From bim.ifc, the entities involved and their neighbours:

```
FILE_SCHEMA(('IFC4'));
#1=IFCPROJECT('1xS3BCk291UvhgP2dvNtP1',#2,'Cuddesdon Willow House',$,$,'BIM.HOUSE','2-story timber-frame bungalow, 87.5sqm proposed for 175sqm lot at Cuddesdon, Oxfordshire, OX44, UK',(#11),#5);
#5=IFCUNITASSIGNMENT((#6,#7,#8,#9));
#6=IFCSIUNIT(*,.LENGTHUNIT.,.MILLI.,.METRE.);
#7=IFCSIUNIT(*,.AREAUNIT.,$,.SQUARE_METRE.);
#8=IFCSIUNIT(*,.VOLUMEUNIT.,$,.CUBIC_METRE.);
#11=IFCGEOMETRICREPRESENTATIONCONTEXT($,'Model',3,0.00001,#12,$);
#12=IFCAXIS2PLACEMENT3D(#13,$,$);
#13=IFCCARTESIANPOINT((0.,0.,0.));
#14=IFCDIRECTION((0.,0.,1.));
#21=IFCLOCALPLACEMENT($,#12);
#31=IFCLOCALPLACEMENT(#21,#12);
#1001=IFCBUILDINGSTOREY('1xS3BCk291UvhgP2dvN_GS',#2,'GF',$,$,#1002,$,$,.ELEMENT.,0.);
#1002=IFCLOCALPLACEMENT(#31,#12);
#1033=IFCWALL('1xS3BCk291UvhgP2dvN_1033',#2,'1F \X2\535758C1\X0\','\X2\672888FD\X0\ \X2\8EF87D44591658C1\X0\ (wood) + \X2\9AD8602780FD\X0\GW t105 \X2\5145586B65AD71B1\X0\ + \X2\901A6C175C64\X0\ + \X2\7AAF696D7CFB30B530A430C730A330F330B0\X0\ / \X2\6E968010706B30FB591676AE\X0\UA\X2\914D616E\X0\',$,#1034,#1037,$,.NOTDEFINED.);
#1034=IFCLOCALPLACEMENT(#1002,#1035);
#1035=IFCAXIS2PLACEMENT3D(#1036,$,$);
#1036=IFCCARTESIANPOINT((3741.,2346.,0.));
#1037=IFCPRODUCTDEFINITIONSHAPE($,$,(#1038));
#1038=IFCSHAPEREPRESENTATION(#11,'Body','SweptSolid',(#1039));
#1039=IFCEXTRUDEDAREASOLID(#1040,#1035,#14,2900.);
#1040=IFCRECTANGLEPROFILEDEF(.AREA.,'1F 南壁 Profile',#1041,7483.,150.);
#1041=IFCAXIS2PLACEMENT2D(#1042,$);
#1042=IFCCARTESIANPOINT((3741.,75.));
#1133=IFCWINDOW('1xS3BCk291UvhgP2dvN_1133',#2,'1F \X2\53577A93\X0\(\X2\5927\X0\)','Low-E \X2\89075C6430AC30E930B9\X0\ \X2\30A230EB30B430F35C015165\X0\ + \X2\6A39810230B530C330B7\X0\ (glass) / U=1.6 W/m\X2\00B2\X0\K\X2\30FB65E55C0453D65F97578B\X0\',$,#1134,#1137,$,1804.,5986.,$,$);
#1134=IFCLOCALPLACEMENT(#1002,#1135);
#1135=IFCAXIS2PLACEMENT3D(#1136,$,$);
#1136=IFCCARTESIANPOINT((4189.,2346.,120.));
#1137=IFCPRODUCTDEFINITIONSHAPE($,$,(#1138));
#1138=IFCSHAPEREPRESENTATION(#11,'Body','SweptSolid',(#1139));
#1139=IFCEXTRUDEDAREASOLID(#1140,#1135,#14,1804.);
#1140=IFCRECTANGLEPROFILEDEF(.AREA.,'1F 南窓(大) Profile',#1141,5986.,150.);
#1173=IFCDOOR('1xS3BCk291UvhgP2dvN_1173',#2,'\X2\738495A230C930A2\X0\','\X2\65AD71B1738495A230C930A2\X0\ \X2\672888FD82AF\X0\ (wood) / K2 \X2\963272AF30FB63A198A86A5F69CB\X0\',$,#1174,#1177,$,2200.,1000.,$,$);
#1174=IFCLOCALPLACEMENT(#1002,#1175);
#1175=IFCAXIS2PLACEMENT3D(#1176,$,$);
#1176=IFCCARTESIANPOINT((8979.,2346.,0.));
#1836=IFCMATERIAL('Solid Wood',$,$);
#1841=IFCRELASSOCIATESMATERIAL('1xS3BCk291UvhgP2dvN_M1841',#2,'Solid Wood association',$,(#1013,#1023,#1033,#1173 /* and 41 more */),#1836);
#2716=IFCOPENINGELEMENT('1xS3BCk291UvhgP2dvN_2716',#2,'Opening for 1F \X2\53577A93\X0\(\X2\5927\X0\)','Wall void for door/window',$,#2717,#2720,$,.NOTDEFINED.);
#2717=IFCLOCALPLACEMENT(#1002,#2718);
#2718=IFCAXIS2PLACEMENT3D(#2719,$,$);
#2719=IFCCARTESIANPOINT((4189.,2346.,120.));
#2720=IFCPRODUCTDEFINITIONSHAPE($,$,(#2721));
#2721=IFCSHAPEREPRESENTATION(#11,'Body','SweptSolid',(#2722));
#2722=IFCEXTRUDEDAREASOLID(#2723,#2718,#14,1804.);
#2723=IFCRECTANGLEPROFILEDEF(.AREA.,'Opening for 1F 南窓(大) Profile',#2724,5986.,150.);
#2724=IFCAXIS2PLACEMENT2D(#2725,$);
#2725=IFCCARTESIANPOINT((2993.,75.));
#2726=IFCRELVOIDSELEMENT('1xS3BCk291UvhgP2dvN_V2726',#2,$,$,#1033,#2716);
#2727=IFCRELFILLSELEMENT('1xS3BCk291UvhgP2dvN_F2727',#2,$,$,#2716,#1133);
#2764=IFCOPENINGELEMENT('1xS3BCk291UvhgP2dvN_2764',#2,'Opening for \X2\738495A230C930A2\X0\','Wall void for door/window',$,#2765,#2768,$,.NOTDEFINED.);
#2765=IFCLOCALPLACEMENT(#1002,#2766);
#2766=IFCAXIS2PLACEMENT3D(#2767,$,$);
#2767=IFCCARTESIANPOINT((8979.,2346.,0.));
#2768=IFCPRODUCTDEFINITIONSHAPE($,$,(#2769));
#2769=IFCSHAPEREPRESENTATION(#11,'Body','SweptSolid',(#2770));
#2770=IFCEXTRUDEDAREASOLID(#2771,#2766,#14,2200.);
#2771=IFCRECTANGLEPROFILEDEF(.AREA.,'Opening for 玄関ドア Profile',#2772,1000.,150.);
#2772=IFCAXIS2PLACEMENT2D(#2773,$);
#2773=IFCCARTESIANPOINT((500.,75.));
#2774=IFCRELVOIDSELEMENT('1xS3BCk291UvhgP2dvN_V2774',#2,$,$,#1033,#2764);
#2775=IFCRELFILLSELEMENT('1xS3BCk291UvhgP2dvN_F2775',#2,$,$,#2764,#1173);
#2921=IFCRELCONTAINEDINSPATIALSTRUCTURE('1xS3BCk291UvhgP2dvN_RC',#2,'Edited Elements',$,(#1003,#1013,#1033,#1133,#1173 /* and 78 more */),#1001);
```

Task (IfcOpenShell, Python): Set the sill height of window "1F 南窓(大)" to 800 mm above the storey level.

```python
import numpy as np
import ifcopenshell
import ifcopenshell.api.geometry
import ifcopenshell.geom
import ifcopenshell.util.element
import ifcopenshell.util.placement
import ifcopenshell.util.shape
import ifcopenshell.util.unit

model = ifcopenshell.open("bim.ifc")
unit_scale = ifcopenshell.util.unit.calculate_unit_scale(model)

window = model.by_guid("1xS3BCk291UvhgP2dvN_1133")
opening = window.FillsVoids[0].RelatingOpeningElement
storey = ifcopenshell.util.element.get_container(window, ifc_class="IfcBuildingStorey")
level = ifcopenshell.util.placement.get_local_placement(storey.ObjectPlacement)[2, 3]

# The opening's origin need not be at the sill, so measure its lowest point.
shape = ifcopenshell.geom.create_shape(ifcopenshell.geom.settings(), opening)
bottom = ifcopenshell.util.shape.get_shape_bottom_elevation(shape, shape.geometry) / unit_scale
dz = level + 0.8 / unit_scale - bottom

shift = np.array([0.0, 0.0, dz])
# The window is not placed relative to its opening, so move both.
for product in (opening, window):
    matrix = ifcopenshell.util.placement.get_local_placement(product.ObjectPlacement)
    matrix[:3, 3] += shift
    ifcopenshell.api.geometry.edit_object_placement(model, product=product, matrix=matrix, is_si=False)

print(f"moved by {dz * unit_scale:+.3f} m")

model.write("bim_updated.ifc")
```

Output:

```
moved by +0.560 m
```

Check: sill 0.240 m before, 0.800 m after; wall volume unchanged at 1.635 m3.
